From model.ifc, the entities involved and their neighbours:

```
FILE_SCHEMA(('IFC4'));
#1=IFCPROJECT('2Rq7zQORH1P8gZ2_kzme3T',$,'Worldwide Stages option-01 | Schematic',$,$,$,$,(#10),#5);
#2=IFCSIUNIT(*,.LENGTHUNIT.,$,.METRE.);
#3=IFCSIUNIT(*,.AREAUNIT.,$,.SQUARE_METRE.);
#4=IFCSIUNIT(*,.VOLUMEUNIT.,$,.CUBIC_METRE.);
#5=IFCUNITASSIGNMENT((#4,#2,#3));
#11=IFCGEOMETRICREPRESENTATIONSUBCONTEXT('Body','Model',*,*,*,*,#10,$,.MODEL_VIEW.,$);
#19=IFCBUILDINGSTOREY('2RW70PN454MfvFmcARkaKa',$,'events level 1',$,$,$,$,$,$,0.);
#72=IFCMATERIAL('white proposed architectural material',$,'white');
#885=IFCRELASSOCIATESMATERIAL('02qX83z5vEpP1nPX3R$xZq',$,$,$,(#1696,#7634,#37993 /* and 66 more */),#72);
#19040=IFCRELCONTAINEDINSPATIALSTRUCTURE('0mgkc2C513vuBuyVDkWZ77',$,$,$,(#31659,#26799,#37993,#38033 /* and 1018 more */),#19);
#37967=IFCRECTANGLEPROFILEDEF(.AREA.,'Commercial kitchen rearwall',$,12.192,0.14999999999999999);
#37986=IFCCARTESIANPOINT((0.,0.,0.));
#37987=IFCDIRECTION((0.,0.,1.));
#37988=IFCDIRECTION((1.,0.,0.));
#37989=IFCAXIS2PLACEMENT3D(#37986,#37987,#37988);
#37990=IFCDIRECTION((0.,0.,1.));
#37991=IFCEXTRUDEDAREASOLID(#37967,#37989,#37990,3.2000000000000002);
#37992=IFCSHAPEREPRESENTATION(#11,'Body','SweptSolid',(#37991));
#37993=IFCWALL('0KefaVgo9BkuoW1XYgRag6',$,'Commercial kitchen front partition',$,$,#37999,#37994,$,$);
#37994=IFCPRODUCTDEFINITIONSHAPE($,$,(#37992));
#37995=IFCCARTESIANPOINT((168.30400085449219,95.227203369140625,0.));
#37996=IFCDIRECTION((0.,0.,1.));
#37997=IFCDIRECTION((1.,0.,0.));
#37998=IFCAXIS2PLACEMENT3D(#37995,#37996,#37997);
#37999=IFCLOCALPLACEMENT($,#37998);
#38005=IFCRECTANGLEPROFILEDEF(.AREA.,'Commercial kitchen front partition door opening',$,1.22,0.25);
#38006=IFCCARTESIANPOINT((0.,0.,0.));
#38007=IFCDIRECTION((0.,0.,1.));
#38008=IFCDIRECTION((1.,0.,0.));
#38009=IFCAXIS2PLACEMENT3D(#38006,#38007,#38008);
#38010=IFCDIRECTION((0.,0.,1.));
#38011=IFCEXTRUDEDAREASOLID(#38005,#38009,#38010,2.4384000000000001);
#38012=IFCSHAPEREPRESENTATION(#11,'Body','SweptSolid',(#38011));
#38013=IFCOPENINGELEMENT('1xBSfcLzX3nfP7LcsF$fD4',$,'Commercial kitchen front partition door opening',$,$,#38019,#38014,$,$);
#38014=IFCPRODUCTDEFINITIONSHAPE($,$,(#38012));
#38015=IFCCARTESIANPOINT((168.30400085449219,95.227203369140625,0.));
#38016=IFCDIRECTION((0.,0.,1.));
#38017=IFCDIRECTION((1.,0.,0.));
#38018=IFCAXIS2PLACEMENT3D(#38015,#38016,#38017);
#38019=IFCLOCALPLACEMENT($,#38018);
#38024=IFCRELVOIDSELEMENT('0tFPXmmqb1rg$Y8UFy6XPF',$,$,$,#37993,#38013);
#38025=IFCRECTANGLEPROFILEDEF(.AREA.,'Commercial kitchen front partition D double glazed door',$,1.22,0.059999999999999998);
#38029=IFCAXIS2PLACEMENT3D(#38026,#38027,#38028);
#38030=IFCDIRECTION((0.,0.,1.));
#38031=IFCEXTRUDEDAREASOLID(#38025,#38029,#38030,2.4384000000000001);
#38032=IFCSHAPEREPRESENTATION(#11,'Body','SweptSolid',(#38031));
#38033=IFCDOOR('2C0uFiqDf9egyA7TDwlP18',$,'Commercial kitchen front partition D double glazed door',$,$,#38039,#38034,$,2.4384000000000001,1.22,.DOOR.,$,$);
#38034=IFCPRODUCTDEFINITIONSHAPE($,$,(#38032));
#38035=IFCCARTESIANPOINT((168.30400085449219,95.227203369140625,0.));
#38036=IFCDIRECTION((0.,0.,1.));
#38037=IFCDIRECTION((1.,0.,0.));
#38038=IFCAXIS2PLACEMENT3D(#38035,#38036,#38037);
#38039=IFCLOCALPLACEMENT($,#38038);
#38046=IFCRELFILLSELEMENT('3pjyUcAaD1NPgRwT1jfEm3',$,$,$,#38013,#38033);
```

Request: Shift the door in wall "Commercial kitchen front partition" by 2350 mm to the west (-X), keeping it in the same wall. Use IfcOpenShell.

```python
import ifcopenshell
import ifcopenshell.api.geometry
import ifcopenshell.util.placement

model = ifcopenshell.open("model.ifc")

door = model.by_id(38033)
opening = door.FillsVoids[0].RelatingOpeningElement
wall = opening.VoidsElements[0].RelatingBuildingElement

wall_matrix = ifcopenshell.util.placement.get_local_placement(wall.ObjectPlacement)
shift = wall_matrix[:3, 0] * -2.35
before = ifcopenshell.util.placement.get_local_placement(door.ObjectPlacement)[:3, 3].copy()

# The door is not placed relative to its opening, so move both.
for product in (opening, door):
    matrix = ifcopenshell.util.placement.get_local_placement(product.ObjectPlacement)
    matrix[:3, 3] += shift
    ifcopenshell.api.geometry.edit_object_placement(model, product=product, matrix=matrix, is_si=False)

after = ifcopenshell.util.placement.get_local_placement(door.ObjectPlacement)[:3, 3]
print("door moved by", (after - before).round(3) + 0.0)

model.write("model_updated.ifc")
```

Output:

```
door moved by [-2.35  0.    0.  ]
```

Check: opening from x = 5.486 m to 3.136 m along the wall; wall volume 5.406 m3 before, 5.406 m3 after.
